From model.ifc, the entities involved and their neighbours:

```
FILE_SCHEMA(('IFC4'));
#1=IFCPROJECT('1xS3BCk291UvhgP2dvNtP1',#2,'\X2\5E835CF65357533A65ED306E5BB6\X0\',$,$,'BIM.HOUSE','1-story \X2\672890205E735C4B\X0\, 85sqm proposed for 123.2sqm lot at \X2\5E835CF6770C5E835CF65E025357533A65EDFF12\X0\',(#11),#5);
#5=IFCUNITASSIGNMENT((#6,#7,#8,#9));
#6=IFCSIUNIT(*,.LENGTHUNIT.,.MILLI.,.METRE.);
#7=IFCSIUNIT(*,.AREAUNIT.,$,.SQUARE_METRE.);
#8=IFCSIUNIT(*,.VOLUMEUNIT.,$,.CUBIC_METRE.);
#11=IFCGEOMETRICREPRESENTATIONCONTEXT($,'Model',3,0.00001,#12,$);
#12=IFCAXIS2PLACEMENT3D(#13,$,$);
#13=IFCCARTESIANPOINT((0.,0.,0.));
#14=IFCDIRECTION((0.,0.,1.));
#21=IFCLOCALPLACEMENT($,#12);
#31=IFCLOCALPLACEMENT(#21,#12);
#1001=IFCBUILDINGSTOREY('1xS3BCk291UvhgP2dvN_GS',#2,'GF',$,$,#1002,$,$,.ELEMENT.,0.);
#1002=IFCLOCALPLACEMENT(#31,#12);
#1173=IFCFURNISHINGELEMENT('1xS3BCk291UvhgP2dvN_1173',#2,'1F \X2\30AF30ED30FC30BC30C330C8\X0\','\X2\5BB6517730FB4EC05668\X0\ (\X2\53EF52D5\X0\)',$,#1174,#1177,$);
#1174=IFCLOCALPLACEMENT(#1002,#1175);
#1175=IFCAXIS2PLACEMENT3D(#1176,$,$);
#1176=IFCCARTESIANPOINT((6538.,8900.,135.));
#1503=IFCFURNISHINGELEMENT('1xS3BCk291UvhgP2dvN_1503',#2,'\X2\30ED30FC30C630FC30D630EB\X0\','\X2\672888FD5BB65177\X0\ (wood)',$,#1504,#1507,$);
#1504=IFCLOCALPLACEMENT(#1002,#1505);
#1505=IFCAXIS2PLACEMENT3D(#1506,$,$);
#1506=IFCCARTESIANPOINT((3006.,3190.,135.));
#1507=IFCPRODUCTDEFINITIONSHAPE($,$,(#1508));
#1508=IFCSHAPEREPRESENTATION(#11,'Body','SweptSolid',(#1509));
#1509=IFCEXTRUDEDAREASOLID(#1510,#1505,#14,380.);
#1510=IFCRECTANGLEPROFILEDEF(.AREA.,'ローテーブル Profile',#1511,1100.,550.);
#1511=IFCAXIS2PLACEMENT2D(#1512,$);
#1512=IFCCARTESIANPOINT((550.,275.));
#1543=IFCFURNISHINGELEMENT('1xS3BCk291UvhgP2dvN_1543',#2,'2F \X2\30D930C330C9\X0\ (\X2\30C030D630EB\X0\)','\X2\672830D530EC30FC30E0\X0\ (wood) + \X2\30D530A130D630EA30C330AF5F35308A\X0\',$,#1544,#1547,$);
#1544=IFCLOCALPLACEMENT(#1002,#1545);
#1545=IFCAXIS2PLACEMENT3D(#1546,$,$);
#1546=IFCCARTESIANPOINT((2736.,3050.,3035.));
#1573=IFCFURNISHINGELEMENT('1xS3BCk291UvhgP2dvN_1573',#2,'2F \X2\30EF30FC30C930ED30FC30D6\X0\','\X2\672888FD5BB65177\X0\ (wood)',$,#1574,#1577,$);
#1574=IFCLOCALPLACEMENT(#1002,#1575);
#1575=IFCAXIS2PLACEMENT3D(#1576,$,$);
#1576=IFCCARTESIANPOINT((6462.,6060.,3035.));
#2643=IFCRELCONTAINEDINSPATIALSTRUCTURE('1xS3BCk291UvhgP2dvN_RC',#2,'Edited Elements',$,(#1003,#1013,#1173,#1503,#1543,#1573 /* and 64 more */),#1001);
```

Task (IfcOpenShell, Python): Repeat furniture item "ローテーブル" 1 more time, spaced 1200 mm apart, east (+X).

```python
import numpy as np
import ifcopenshell
import ifcopenshell.api.geometry
import ifcopenshell.api.root
import ifcopenshell.util.element
import ifcopenshell.util.placement
import ifcopenshell.util.unit

model = ifcopenshell.open("model.ifc")
unit_scale = ifcopenshell.util.unit.calculate_unit_scale(model)


def reuse_history(source, copy):
    """copy_class also copies each property set's owner history, people and application; keep the originals."""
    for rel in copy.IsDefinedBy:
        if rel.is_a("IfcRelDefinesByProperties") and (history := rel.RelatingPropertyDefinition.OwnerHistory):
            rel.RelatingPropertyDefinition.OwnerHistory = source.OwnerHistory
            ifcopenshell.util.element.remove_deep2(model, history)


source = model.by_guid("1xS3BCk291UvhgP2dvN_1503")
base = ifcopenshell.util.placement.get_local_placement(source.ObjectPlacement)
step = np.array([1.0, 0.0, 0.0]) * 1.2 / unit_scale

for i in range(1, 2):
    copy = ifcopenshell.api.root.copy_class(model, product=source)
    copy.Representation = ifcopenshell.util.element.copy_deep(
        model, source.Representation, exclude=["IfcGeometricRepresentationContext", "IfcRepresentationMap"]
    )
    reuse_history(source, copy)
    matrix = base.copy()
    matrix[:3, 3] += i * step
    print("added at", matrix[:3, 3].round(3) + 0.0)
    ifcopenshell.api.geometry.edit_object_placement(model, product=copy, matrix=matrix, is_si=False)

model.write("model_rev.ifc")
```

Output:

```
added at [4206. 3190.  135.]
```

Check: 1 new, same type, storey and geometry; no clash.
